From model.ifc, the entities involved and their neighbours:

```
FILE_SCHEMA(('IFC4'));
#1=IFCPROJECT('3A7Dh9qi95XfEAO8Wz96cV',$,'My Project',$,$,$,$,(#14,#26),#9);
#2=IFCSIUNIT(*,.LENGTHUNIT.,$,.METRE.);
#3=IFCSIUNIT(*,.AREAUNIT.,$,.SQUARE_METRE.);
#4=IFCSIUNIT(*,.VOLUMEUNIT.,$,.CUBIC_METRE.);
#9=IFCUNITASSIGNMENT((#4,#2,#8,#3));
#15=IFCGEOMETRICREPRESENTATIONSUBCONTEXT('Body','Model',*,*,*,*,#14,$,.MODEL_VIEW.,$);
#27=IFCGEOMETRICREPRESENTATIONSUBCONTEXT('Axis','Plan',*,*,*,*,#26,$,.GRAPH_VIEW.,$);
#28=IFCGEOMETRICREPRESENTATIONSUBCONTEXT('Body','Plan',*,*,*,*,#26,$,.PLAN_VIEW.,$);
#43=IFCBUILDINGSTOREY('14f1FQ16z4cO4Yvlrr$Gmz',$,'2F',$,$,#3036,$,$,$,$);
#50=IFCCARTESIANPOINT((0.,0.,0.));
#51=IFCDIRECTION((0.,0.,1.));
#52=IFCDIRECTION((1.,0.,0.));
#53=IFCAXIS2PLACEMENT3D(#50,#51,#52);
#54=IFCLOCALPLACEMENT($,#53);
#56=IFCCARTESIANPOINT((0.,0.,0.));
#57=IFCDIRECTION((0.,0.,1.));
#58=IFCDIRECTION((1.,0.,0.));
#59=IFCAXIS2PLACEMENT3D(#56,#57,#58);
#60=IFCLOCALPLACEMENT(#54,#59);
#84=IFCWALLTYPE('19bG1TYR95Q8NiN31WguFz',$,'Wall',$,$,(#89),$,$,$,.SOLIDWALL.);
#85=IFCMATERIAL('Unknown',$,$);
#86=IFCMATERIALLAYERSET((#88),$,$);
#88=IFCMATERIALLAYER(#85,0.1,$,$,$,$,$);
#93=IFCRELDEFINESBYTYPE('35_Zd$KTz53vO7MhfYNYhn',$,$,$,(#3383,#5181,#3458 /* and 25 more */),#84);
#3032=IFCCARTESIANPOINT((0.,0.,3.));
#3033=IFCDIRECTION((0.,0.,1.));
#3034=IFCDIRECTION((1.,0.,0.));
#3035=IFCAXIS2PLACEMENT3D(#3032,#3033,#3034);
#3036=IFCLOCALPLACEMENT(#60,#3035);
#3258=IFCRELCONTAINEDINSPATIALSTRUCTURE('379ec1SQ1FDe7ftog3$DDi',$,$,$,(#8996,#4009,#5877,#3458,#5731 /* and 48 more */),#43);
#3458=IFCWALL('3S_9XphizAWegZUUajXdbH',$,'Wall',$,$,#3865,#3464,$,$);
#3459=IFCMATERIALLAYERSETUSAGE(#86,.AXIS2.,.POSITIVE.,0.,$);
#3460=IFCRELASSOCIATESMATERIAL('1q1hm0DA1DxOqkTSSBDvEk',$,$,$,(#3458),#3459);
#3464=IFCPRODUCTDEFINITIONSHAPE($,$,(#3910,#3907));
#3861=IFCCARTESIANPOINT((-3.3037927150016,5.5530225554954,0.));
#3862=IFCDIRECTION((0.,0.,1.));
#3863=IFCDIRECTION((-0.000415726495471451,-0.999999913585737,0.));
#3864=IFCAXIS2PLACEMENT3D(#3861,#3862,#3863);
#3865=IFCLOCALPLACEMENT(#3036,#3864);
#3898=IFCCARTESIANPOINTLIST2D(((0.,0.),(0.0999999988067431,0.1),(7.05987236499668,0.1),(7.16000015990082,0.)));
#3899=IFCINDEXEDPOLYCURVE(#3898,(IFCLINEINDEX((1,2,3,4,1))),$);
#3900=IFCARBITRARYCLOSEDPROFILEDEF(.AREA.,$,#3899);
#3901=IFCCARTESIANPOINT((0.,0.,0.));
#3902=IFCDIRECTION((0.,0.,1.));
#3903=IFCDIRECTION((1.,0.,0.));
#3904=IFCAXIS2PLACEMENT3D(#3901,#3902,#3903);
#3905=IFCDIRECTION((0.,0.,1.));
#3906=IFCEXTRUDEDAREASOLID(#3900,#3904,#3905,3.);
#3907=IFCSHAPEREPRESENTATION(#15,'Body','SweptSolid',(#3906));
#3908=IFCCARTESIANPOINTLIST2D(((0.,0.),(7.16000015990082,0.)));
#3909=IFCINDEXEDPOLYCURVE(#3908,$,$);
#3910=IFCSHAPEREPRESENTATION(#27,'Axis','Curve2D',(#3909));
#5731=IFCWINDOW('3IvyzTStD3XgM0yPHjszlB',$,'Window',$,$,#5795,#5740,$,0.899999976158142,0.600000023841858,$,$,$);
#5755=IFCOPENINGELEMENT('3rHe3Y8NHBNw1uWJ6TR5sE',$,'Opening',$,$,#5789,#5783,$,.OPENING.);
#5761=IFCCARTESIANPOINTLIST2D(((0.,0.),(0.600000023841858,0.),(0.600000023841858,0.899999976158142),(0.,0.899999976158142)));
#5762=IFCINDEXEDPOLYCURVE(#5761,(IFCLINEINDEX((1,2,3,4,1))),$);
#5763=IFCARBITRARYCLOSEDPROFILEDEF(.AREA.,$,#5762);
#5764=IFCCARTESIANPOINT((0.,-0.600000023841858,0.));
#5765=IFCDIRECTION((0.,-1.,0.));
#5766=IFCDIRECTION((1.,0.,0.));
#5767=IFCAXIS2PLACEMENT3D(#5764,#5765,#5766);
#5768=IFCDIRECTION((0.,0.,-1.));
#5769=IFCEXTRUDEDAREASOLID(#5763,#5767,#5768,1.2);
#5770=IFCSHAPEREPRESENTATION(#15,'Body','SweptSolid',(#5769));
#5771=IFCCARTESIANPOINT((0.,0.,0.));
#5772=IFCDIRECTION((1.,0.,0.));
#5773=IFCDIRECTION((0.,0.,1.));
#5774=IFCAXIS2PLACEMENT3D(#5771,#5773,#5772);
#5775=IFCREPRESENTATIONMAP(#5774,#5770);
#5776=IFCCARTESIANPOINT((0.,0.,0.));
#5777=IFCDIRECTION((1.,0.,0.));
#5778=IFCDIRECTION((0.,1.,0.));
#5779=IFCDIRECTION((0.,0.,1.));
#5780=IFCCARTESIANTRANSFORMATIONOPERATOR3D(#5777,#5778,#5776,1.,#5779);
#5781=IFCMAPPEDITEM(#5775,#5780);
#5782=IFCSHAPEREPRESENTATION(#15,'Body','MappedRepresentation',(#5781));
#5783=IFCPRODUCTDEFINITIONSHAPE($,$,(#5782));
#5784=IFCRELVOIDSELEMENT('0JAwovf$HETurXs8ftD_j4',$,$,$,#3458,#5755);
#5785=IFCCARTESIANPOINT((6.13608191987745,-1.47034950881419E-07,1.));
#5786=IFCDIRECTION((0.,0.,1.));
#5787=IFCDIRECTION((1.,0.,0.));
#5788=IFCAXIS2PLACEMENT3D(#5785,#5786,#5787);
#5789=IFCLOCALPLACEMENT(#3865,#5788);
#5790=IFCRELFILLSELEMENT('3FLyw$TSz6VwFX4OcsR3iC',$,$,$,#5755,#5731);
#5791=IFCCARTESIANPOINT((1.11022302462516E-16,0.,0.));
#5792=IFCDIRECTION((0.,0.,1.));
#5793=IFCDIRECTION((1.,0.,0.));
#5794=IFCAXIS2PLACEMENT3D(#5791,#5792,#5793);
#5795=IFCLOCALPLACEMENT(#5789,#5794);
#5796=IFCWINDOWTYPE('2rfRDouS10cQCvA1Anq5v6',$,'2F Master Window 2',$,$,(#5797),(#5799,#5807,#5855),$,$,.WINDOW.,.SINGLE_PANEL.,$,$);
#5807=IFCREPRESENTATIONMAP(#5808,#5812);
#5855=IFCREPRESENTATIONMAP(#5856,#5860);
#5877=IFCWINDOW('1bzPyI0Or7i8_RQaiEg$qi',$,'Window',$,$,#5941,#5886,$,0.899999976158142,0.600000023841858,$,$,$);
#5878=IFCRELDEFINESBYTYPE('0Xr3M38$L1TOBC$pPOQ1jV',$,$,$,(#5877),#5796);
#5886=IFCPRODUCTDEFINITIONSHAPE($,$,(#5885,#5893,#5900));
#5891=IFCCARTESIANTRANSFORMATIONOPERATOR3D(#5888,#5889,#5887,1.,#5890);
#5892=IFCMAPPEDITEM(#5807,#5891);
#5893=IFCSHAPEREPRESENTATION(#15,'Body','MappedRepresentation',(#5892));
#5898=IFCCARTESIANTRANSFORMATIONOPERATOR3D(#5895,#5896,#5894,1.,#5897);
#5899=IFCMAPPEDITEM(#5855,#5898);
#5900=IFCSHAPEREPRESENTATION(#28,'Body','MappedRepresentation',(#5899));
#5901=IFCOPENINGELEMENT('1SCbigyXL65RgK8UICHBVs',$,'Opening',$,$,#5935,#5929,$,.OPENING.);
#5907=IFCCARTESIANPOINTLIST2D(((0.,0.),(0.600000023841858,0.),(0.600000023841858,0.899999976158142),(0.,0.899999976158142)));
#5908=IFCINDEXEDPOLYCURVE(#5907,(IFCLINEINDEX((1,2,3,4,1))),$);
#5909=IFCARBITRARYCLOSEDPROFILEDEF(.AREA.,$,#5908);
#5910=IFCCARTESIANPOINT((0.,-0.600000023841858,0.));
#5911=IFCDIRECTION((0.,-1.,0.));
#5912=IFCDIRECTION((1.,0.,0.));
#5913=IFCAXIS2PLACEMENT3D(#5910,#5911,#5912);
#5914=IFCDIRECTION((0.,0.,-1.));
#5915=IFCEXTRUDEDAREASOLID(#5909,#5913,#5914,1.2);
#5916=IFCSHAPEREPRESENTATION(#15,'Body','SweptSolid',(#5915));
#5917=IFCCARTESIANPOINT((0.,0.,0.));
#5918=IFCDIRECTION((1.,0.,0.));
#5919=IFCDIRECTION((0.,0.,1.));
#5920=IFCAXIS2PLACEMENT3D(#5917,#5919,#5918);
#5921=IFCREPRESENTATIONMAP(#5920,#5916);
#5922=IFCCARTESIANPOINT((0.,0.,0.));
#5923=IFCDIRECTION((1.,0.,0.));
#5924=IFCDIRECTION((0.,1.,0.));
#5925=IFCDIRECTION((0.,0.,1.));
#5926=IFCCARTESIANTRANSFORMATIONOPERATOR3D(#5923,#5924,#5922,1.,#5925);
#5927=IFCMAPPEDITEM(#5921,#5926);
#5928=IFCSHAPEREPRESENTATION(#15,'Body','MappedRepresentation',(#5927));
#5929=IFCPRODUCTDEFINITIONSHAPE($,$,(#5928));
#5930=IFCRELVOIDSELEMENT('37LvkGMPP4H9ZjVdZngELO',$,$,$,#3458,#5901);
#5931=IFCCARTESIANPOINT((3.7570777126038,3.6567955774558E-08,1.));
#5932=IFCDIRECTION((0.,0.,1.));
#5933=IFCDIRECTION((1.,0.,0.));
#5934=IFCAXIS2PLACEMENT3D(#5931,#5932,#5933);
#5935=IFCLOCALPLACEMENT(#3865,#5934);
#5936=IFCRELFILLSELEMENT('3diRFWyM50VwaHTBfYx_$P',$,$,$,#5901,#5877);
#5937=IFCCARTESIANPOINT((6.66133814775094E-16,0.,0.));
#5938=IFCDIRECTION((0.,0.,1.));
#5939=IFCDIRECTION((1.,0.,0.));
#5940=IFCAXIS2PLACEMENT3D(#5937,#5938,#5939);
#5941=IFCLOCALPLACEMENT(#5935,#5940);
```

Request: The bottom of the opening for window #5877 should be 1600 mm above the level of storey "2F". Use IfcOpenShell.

```python
import numpy as np
import ifcopenshell
import ifcopenshell.api.geometry
import ifcopenshell.geom
import ifcopenshell.util.element
import ifcopenshell.util.placement
import ifcopenshell.util.shape
import ifcopenshell.util.unit

model = ifcopenshell.open("model.ifc")
unit_scale = ifcopenshell.util.unit.calculate_unit_scale(model)

window = model.by_guid("1bzPyI0Or7i8_RQaiEg$qi")
opening = window.FillsVoids[0].RelatingOpeningElement
storey = ifcopenshell.util.element.get_container(window, ifc_class="IfcBuildingStorey")
level = ifcopenshell.util.placement.get_local_placement(storey.ObjectPlacement)[2, 3]

# The opening's origin need not be at the sill, so measure its lowest point.
shape = ifcopenshell.geom.create_shape(ifcopenshell.geom.settings(), opening)
bottom = ifcopenshell.util.shape.get_shape_bottom_elevation(shape, shape.geometry) / unit_scale
dz = level + 1.6 - bottom

shift = np.array([0.0, 0.0, dz])
# The window is placed relative to its opening, so it follows when the opening moves.
matrix = ifcopenshell.util.placement.get_local_placement(opening.ObjectPlacement)
matrix[:3, 3] += shift
ifcopenshell.api.geometry.edit_object_placement(
    model, product=opening, matrix=matrix, is_si=False, should_transform_children=True
)

print(f"moved by {dz * unit_scale:+.3f} m")

model.write("model-out.ifc")
```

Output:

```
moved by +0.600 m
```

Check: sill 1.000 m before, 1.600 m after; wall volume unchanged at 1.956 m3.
